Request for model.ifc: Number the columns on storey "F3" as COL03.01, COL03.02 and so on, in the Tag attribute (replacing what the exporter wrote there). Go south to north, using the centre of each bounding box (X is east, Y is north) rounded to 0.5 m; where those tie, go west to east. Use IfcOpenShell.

First a look at what the model holds.

```python
import ifcopenshell
import ifcopenshell.util.element
import ifcopenshell.util.placement

model = ifcopenshell.open("model.ifc")
print(model.schema)
storey = next(s for s in model.by_type("IfcBuildingStorey") if s.Name == "F3")
columns = [e for e in ifcopenshell.util.element.get_decomposition(storey) if e.is_a("IfcColumn")]
for e in sorted(columns, key=lambda e: e.id()):
    origin = ifcopenshell.util.placement.get_local_placement(e.ObjectPlacement)[:3, 3]
    print(e.id(), e.Tag, e.Name, origin.round(2) + 0.0, sep=" | ")
```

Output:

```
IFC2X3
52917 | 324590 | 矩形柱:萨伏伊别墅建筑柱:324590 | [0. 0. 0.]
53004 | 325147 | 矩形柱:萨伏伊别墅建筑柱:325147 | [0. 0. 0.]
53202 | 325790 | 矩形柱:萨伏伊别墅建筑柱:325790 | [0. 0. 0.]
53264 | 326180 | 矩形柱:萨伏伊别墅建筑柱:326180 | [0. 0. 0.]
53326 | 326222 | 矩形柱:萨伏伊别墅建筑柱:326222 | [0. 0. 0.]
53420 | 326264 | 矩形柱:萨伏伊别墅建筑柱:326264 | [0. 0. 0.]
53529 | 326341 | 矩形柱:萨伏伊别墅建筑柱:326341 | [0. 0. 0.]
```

```python
import ifcopenshell
import ifcopenshell.geom
import ifcopenshell.util.element
import ifcopenshell.util.shape

model = ifcopenshell.open("model.ifc")
settings = ifcopenshell.geom.settings()
settings.set("use-world-coords", True)


def centre(element):
    shape = ifcopenshell.geom.create_shape(settings, element)
    return ifcopenshell.util.shape.get_bbox_centroid(shape.geometry)


storey = next(s for s in model.by_type("IfcBuildingStorey") if s.Name == "F3")
columns = [e for e in ifcopenshell.util.element.get_decomposition(storey) if e.is_a("IfcColumn")]

# Insertion points can sit at a corner or the storey origin, so sort by the geometry (in metres).
centres = {e: centre(e) for e in columns}
columns.sort(key=lambda e: (round(centres[e][1] / 0.5), centres[e][0]))

for i, e in enumerate(columns, start=1):
    number = f"COL03.{i:02d}"
    e.Tag = number
    print(e.id(), number)

model.write("model_updated.ifc")
```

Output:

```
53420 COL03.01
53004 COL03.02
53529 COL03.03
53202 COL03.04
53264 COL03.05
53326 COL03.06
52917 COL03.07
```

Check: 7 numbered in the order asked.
